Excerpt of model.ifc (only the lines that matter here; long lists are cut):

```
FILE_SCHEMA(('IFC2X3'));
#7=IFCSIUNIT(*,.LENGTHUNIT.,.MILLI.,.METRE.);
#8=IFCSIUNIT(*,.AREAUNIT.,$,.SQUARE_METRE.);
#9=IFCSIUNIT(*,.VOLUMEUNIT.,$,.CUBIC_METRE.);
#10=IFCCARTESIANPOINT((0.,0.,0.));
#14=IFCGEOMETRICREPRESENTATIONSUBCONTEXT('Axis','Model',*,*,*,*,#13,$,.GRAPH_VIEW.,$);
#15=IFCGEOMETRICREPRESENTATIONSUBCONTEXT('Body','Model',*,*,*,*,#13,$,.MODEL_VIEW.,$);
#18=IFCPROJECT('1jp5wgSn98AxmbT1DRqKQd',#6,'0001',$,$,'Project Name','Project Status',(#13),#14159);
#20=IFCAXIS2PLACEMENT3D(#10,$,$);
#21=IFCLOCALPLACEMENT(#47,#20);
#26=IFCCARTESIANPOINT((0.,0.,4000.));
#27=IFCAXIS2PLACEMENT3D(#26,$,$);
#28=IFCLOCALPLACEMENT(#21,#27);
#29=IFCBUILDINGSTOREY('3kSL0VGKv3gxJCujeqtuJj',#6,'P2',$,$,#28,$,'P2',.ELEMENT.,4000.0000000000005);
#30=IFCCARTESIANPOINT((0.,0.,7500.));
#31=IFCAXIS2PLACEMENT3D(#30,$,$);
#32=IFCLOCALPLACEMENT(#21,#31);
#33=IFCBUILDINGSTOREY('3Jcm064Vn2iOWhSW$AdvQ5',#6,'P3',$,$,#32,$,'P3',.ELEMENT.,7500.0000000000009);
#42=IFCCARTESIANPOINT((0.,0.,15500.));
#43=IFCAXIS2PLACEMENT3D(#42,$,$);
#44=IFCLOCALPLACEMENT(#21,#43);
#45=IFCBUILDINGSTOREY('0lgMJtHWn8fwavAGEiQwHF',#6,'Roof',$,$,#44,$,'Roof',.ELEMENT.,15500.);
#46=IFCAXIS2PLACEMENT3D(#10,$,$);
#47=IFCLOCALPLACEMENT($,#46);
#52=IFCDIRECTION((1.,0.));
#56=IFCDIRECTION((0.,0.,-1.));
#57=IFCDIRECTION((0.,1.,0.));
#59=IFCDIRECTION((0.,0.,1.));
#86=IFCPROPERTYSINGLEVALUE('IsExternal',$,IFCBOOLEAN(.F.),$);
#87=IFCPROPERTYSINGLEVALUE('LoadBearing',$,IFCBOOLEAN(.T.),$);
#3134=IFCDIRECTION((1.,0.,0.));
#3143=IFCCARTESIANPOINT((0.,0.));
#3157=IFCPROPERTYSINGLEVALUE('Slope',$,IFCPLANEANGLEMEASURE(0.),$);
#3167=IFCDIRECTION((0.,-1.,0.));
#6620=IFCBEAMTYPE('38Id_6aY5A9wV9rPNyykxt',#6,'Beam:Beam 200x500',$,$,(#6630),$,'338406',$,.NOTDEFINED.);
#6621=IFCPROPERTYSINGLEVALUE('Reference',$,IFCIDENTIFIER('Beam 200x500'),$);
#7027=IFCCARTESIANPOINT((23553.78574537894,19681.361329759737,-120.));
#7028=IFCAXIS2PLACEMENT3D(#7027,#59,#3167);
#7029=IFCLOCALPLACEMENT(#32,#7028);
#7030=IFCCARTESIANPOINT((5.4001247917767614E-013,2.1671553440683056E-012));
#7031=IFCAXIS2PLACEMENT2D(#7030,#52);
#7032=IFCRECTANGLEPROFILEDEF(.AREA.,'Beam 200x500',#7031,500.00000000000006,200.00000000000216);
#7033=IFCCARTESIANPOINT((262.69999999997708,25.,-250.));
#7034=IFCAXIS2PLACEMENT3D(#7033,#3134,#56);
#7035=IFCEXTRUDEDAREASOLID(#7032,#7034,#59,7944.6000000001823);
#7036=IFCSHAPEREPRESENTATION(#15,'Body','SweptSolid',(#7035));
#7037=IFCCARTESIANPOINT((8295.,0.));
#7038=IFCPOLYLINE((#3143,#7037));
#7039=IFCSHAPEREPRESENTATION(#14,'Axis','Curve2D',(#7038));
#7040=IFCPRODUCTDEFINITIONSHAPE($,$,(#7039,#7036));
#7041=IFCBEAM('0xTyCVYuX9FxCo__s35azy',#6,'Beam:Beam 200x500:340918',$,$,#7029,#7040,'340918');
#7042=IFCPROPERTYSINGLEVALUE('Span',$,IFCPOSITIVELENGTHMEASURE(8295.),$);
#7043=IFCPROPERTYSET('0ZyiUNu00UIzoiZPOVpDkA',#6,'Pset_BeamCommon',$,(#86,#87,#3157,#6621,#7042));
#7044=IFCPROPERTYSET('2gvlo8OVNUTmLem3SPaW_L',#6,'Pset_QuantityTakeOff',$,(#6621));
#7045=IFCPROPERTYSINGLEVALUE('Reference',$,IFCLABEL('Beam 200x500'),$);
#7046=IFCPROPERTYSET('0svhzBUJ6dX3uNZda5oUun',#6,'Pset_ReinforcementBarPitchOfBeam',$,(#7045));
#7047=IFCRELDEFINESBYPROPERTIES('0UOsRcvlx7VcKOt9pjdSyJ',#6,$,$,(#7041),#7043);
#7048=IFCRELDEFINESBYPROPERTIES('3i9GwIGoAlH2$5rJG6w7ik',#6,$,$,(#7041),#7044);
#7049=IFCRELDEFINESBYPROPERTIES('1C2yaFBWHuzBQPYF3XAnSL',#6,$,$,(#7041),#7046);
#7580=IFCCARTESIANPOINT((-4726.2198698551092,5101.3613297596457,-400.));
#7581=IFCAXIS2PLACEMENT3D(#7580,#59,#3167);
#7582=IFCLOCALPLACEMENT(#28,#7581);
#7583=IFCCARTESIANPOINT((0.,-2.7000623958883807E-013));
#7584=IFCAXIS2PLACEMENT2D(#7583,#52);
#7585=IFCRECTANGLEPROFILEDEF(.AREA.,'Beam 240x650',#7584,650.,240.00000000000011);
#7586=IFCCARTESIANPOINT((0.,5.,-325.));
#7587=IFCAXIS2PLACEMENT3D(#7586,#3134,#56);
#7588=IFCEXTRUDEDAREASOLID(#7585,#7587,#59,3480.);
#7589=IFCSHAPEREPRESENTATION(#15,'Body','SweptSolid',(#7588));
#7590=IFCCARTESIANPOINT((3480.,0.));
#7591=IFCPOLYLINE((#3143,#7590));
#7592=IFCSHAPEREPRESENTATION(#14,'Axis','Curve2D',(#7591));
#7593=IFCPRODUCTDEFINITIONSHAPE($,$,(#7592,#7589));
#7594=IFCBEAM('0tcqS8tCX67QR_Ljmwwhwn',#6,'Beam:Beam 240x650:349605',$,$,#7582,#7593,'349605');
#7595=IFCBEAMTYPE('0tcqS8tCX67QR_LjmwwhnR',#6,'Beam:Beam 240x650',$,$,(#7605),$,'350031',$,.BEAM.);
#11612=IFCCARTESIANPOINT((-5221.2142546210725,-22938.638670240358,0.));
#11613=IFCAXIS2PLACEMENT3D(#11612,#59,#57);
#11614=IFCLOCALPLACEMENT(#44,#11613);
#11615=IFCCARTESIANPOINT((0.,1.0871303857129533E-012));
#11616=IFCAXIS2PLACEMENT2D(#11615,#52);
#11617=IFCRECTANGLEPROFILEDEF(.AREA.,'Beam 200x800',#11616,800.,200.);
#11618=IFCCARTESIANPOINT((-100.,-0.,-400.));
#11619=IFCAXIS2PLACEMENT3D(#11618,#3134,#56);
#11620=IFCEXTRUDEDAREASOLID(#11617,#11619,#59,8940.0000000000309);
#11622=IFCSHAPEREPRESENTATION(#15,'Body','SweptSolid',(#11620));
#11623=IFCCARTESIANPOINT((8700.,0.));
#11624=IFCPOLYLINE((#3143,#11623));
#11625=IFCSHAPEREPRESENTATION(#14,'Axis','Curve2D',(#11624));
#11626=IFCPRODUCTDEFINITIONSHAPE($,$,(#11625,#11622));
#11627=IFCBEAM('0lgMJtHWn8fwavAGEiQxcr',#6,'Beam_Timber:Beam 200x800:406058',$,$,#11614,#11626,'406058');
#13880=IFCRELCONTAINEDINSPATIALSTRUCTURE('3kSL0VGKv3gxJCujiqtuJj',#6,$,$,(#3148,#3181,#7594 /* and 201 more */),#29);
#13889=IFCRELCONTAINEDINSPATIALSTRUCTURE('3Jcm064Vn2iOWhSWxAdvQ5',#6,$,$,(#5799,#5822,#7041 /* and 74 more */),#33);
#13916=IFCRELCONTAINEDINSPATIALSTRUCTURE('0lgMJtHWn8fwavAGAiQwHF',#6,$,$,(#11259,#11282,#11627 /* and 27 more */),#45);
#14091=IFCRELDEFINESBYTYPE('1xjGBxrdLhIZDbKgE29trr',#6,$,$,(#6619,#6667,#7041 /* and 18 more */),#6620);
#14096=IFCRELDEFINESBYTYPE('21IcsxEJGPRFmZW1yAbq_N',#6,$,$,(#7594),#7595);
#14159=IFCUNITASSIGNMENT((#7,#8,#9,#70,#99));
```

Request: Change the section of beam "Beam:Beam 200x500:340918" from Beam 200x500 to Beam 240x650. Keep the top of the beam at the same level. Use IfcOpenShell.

```python
import ifcopenshell
import ifcopenshell.api.pset
import ifcopenshell.api.type
import ifcopenshell.util.element
import ifcopenshell.util.representation

model = ifcopenshell.open("model.ifc")

member = model.by_id(7041)
source = next(p for p in model.by_type("IfcRectangleProfileDef") if p.ProfileName == "Beam 240x650")

body = ifcopenshell.util.representation.get_representation(member, "Model", "Body")
solid = body.Items[0]
old_profile = solid.SweptArea

# Copy the section's sizes but keep this member's own profile position.
profile = ifcopenshell.util.element.copy(model, source)
# Profiles are centred, so shift by half the change in depth to hold the top.
shift = (old_profile.XDim - profile.XDim) / 2
x, y = old_profile.Position.Location.Coordinates
up = (-1.0, 0.0)  # upwards, in the solid's own plane
location = model.createIfcCartesianPoint((x + up[0] * shift, y + up[1] * shift))
profile.Position = model.createIfcAxis2Placement2D(location, old_profile.Position.RefDirection)
solid.SweptArea = profile
if not model.get_total_inverses(old_profile):
    ifcopenshell.util.element.remove_deep2(model, old_profile)

new_type = model.by_guid("0tcqS8tCX67QR_LjmwwhnR")
ifcopenshell.api.type.assign_type(
    model, related_objects=[member], relating_type=new_type, should_map_representations=False
)
member.Name = member.Name.replace("Beam 200x500", "Beam 240x650")
pset = model.by_id(ifcopenshell.util.element.get_pset(member, "Pset_BeamCommon", should_inherit=False)["id"])
ifcopenshell.api.pset.edit_pset(model, pset=pset, properties={"Reference": "Beam 240x650"})
pset = model.by_id(ifcopenshell.util.element.get_pset(member, "Pset_QuantityTakeOff", should_inherit=False)["id"])
ifcopenshell.api.pset.edit_pset(model, pset=pset, properties={"Reference": "Beam 240x650"})
pset = model.by_id(ifcopenshell.util.element.get_pset(member, "Pset_ReinforcementBarPitchOfBeam", should_inherit=False)["id"])
ifcopenshell.api.pset.edit_pset(model, pset=pset, properties={"Reference": "Beam 240x650"})

print(solid.SweptArea)

model.write("model_edited.ifc")
```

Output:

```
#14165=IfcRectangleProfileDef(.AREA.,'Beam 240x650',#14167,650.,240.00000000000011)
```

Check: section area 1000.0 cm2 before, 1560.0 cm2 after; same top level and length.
